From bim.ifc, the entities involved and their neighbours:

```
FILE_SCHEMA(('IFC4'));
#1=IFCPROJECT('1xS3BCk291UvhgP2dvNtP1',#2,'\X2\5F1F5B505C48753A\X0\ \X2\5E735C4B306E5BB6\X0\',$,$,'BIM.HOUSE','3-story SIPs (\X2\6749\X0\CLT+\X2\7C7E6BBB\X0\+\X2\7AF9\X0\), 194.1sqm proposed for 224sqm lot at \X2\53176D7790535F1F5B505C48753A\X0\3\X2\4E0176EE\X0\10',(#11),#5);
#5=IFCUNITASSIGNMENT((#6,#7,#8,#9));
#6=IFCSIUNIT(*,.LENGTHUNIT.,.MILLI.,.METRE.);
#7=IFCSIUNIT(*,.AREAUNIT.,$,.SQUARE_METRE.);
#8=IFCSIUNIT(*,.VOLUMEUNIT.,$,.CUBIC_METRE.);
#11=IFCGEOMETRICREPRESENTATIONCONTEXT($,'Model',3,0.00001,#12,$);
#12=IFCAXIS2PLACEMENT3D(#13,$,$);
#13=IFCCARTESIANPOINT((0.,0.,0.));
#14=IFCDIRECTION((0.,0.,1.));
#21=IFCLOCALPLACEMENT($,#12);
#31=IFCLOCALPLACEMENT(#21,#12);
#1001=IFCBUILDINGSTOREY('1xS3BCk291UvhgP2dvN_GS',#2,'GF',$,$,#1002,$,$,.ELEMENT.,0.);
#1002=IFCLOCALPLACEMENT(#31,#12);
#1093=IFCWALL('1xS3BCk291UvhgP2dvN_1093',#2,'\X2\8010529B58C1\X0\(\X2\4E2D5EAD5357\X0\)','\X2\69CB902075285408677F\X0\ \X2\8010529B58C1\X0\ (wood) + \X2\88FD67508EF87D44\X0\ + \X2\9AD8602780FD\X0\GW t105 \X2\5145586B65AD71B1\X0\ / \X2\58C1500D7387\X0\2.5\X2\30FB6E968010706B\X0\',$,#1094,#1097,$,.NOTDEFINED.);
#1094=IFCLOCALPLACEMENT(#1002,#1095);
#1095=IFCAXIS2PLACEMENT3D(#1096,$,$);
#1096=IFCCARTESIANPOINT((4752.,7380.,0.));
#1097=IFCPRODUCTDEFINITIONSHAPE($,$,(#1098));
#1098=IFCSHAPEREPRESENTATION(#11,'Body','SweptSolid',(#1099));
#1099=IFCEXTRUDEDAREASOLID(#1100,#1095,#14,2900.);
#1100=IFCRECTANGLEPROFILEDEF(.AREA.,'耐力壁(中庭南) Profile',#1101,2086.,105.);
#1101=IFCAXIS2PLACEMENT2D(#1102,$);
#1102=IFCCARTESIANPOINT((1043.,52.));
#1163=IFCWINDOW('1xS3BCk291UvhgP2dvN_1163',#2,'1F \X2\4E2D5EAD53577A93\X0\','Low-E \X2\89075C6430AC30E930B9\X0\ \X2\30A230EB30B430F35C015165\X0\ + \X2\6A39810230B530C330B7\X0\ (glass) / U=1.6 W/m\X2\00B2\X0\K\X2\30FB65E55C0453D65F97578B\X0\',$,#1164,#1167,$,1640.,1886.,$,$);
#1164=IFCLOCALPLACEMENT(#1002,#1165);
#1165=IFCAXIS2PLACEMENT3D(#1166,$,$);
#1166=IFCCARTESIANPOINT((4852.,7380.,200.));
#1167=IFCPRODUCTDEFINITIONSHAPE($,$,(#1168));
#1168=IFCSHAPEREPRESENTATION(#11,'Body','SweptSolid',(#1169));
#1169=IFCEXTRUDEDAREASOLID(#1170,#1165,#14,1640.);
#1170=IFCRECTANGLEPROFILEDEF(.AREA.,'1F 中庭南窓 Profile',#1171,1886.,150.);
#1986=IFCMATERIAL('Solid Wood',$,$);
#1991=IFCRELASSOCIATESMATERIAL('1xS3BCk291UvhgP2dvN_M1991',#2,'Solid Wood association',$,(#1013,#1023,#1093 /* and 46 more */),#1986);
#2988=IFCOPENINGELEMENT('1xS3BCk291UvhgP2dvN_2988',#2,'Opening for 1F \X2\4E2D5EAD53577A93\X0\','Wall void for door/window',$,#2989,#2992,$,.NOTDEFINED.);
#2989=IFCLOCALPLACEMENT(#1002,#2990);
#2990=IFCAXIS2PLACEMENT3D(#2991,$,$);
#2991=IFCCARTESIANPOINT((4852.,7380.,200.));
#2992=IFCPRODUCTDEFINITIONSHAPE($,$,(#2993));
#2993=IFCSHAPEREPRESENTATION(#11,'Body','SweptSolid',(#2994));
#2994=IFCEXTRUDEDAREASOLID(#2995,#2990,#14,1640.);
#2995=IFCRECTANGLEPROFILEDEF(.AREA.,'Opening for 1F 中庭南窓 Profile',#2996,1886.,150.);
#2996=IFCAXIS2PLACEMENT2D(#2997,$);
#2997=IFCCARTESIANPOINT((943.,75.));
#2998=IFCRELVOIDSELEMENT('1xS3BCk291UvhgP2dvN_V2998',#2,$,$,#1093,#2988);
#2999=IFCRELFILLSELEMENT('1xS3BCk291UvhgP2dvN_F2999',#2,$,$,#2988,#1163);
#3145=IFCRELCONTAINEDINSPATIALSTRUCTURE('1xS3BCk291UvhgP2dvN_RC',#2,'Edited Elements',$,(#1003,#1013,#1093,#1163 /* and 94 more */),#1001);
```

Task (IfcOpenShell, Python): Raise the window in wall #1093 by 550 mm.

```python
import numpy as np
import ifcopenshell
import ifcopenshell.api.geometry
import ifcopenshell.util.placement
import ifcopenshell.util.unit

model = ifcopenshell.open("bim.ifc")
unit_scale = ifcopenshell.util.unit.calculate_unit_scale(model)

window = model.by_guid("1xS3BCk291UvhgP2dvN_1163")
opening = window.FillsVoids[0].RelatingOpeningElement
dz = 0.55 / unit_scale

shift = np.array([0.0, 0.0, dz])
# The window is not placed relative to its opening, so move both.
for product in (opening, window):
    matrix = ifcopenshell.util.placement.get_local_placement(product.ObjectPlacement)
    matrix[:3, 3] += shift
    ifcopenshell.api.geometry.edit_object_placement(model, product=product, matrix=matrix, is_si=False)

print(f"moved by {dz * unit_scale:+.3f} m")

model.write("bim_edited.ifc")
```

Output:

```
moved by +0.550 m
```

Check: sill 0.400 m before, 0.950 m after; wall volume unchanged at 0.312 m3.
